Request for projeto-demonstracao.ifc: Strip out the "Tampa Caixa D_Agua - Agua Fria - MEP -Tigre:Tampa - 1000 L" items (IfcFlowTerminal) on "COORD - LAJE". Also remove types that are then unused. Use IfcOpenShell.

First a look at what the model holds.

```python
import ifcopenshell
import ifcopenshell.util.element

model = ifcopenshell.open("projeto-demonstracao.ifc")
print(model.schema)
storey = next(s for s in model.by_type("IfcBuildingStorey") if s.Name == "COORD - LAJE")
terminals = [e for e in ifcopenshell.util.element.get_decomposition(storey) if e.is_a("IfcFlowTerminal")]
seen = {}
for e in terminals:
    element_type = ifcopenshell.util.element.get_type(e)
    name = element_type.Name if element_type not in (None, e) else None
    seen[name] = seen.get(name, 0) + 1
for name, count in sorted(seen.items(), key=str):
    print(count, "x", name)
```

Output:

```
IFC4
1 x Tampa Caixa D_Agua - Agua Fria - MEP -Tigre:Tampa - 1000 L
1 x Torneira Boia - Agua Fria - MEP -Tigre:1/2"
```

```python
import ifcopenshell
import ifcopenshell.api.root
import ifcopenshell.util.element

model = ifcopenshell.open("projeto-demonstracao.ifc")

storey = next(s for s in model.by_type("IfcBuildingStorey") if s.Name == "COORD - LAJE")
terminals = [e for e in ifcopenshell.util.element.get_decomposition(storey) if e.is_a("IfcFlowTerminal")]
targets = [e for e in terminals if (t := ifcopenshell.util.element.get_type(e)) not in (None, e) and t.Name == "Tampa Caixa D_Agua - Agua Fria - MEP -Tigre:Tampa - 1000 L"]
types = {ifcopenshell.util.element.get_type(e) for e in targets} - {None, *targets}

for e in targets:
    ifcopenshell.api.root.remove_product(model, product=e)
print(len(targets), "removed")

unused = [t for t in types if not ifcopenshell.util.element.get_types(t)]
for t in unused:
    ifcopenshell.api.root.remove_product(model, product=t)
print(len(unused), "unused types removed")

model.write("projeto-demonstracao_rev.ifc")
```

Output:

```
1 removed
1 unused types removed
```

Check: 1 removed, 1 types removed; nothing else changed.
